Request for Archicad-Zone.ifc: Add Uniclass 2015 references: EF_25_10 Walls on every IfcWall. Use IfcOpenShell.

First a look at what the model holds.

```python
import ifcopenshell

model = ifcopenshell.open("Archicad-Zone.ifc")
print(model.schema)
print("classifications:", [c.Name for c in model.by_type("IfcClassification")])
for ifc_class in ("IfcDoor", "IfcRoof", "IfcStair", "IfcWall", "IfcWindow"):
    print(ifc_class, len(model.by_type(ifc_class)))
```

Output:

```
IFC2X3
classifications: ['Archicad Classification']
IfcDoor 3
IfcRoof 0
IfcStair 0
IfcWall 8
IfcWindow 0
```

```python
import ifcopenshell
import ifcopenshell.api.classification

model = ifcopenshell.open("Archicad-Zone.ifc")

# IFC2X3 requires Source and Edition and has no link from the project to the system.
system = model.create_entity("IfcClassification", Source="NBS", Edition="2015", Name="Uniclass 2015")

codes = {
    "IfcWall": ("EF_25_10", "Walls"),
}
for ifc_class, (code, name) in codes.items():
    products = model.by_type(ifc_class)
    ifcopenshell.api.classification.add_reference(
        model, products=products, classification=system, identification=code, name=name
    )
    print(code, len(products))

model.write("Archicad-Zone-out.ifc")
```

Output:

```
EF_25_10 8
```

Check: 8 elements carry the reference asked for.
